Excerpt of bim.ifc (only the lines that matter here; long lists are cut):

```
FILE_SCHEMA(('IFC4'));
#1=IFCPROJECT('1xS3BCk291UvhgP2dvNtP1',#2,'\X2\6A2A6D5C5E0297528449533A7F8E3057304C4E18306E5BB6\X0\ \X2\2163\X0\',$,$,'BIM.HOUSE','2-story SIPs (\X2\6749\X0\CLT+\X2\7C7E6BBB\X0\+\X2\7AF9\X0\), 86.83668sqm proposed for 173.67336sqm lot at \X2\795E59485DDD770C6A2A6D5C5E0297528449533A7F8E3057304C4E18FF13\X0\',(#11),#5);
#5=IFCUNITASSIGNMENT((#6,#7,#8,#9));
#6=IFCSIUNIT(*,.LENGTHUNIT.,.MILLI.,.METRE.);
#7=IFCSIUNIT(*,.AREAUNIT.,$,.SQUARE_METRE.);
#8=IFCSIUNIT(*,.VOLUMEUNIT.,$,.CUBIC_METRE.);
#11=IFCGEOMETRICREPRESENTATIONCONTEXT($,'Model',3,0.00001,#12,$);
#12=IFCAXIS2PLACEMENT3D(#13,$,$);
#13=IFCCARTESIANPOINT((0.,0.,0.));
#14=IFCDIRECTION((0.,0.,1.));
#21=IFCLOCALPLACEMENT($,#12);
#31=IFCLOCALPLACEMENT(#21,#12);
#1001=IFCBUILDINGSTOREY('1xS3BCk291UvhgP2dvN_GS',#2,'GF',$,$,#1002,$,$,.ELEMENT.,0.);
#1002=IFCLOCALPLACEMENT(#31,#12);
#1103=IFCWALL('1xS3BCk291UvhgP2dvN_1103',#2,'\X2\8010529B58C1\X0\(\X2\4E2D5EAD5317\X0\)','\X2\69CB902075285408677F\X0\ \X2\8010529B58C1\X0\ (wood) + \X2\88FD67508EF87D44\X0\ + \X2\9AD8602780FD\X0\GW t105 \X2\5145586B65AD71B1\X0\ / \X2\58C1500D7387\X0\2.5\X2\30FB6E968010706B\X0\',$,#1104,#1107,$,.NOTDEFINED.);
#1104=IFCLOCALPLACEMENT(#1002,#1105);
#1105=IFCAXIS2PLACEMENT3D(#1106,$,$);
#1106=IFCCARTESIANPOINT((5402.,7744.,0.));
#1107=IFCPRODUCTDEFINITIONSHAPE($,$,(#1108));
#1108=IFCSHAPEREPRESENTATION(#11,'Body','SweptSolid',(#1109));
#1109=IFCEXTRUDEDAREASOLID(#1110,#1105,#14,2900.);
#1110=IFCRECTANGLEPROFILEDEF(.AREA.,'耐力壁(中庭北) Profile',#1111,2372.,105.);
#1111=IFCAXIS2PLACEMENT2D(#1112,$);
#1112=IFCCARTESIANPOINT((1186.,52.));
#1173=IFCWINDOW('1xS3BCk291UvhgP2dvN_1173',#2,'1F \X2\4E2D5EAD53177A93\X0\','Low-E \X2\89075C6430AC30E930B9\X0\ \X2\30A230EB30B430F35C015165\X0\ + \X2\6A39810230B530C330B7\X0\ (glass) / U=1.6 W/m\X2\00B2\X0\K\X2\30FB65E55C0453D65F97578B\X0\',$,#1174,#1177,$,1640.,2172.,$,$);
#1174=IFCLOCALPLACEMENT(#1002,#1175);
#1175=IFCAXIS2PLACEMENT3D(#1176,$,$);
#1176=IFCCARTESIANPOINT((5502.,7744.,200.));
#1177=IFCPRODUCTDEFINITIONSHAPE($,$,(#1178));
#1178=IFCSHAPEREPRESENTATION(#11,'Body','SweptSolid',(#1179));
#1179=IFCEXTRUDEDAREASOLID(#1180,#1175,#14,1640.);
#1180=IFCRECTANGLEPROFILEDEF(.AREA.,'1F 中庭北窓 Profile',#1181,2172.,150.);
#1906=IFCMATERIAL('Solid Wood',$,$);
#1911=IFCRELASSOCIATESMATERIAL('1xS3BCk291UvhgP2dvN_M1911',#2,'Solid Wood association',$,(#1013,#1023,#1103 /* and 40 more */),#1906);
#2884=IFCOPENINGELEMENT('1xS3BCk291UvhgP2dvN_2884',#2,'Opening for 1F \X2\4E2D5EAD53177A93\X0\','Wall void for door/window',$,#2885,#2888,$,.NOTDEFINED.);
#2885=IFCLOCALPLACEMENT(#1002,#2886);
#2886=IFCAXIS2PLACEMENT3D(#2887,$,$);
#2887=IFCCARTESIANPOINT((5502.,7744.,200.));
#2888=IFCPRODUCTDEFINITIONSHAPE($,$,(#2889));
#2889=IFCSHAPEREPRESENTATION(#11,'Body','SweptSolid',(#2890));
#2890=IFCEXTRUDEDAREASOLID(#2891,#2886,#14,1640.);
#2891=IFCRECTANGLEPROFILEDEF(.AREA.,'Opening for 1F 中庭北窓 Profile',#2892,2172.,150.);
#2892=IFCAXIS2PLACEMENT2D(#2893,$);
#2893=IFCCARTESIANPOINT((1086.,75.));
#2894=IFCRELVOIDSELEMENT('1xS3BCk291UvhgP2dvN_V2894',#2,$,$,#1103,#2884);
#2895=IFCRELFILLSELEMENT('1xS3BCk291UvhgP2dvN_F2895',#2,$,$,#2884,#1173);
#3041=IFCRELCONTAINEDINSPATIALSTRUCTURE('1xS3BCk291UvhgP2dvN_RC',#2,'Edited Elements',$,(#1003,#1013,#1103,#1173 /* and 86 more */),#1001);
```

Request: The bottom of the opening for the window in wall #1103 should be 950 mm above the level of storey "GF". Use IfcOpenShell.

```python
import numpy as np
import ifcopenshell
import ifcopenshell.api.geometry
import ifcopenshell.geom
import ifcopenshell.util.element
import ifcopenshell.util.placement
import ifcopenshell.util.shape
import ifcopenshell.util.unit

model = ifcopenshell.open("bim.ifc")
unit_scale = ifcopenshell.util.unit.calculate_unit_scale(model)

window = model.by_guid("1xS3BCk291UvhgP2dvN_1173")
opening = window.FillsVoids[0].RelatingOpeningElement
storey = ifcopenshell.util.element.get_container(window, ifc_class="IfcBuildingStorey")
level = ifcopenshell.util.placement.get_local_placement(storey.ObjectPlacement)[2, 3]

# The opening's origin need not be at the sill, so measure its lowest point.
shape = ifcopenshell.geom.create_shape(ifcopenshell.geom.settings(), opening)
bottom = ifcopenshell.util.shape.get_shape_bottom_elevation(shape, shape.geometry) / unit_scale
dz = level + 0.95 / unit_scale - bottom

shift = np.array([0.0, 0.0, dz])
# The window is not placed relative to its opening, so move both.
for product in (opening, window):
    matrix = ifcopenshell.util.placement.get_local_placement(product.ObjectPlacement)
    matrix[:3, 3] += shift
    ifcopenshell.api.geometry.edit_object_placement(model, product=product, matrix=matrix, is_si=False)

print(f"moved by {dz * unit_scale:+.3f} m")

model.write("bim-out.ifc")
```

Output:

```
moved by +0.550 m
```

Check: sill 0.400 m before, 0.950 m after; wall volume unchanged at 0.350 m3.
